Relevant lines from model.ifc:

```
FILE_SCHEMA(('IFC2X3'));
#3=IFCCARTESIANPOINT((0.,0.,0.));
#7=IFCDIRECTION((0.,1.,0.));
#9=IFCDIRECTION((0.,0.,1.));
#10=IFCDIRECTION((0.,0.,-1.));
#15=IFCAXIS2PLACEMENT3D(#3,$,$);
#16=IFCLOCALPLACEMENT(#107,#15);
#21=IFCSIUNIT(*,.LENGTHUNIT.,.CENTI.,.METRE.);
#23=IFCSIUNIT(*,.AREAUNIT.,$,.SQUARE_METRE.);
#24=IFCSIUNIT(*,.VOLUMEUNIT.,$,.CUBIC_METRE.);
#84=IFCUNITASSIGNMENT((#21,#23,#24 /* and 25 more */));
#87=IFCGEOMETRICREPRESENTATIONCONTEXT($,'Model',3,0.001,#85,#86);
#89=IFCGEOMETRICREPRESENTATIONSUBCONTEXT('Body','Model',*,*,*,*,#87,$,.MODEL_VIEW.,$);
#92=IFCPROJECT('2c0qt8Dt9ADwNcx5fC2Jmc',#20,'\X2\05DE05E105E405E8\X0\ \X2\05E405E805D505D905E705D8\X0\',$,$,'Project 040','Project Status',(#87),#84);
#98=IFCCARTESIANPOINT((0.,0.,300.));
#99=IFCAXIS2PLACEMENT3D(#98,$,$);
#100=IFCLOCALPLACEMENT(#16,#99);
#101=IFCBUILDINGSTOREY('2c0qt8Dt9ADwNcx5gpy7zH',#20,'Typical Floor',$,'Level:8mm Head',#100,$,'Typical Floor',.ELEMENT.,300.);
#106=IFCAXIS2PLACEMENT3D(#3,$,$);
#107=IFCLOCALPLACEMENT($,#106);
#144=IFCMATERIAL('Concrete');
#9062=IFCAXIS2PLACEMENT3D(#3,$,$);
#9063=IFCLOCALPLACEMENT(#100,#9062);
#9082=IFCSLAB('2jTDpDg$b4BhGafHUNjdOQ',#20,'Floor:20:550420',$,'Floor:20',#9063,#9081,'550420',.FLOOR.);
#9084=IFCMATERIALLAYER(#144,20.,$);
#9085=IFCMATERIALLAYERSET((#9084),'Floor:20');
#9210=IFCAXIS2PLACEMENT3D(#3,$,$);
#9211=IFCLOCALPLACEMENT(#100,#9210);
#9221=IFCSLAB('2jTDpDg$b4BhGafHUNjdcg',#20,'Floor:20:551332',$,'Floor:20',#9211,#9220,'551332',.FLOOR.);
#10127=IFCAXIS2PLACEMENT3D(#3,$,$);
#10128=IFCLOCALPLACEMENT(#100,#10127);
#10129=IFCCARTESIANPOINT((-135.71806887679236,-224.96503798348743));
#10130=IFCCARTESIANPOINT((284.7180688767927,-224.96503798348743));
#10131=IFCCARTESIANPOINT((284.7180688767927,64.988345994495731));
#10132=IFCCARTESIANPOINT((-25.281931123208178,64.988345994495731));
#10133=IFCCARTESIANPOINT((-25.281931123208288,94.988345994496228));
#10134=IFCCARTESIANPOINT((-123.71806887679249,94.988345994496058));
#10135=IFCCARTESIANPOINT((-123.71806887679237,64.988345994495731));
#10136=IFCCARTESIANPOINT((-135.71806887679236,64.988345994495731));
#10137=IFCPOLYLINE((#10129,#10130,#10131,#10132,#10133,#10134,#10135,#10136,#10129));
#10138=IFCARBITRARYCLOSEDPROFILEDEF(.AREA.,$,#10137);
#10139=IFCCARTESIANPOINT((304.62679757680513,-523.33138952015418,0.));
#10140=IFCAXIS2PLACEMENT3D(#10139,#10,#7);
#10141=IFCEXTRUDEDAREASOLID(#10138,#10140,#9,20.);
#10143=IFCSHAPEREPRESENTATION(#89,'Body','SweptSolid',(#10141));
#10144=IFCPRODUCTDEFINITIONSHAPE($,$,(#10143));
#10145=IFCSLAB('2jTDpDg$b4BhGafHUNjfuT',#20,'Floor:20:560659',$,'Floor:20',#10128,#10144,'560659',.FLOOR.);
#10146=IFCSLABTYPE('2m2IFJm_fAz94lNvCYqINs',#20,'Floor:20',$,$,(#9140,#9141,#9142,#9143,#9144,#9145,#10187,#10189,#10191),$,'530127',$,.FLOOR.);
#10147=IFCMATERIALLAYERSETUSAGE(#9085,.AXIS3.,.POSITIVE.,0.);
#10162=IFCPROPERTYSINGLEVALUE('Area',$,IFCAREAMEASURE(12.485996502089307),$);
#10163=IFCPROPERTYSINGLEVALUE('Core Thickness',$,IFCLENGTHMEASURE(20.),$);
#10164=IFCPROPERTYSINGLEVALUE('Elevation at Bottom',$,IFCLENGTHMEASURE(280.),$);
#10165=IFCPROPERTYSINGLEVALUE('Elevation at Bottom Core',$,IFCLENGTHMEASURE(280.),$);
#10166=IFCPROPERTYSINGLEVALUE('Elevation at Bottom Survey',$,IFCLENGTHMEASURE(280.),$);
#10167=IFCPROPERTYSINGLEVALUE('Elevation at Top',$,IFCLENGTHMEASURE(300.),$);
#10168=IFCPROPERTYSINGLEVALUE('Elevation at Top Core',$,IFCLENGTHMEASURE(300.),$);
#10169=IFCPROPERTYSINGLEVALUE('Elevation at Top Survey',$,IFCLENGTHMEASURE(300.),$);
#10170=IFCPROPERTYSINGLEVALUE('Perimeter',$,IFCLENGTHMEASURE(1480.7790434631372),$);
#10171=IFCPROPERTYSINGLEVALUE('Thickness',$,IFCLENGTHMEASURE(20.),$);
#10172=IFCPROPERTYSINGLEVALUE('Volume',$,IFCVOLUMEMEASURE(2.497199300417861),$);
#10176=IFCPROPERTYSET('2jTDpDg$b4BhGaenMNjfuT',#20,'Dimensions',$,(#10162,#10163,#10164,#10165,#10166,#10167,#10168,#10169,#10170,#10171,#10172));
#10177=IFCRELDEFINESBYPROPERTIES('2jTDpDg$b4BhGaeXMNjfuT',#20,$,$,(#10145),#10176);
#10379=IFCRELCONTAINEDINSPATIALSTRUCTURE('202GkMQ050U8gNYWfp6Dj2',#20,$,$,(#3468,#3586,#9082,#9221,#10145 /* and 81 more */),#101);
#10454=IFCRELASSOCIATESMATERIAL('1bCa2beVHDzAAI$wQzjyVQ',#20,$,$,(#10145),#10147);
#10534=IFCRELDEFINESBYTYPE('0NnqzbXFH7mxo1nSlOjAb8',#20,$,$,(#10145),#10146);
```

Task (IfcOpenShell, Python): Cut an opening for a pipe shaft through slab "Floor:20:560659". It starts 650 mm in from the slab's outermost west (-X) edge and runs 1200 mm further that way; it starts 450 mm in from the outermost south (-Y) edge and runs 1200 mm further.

```python
import numpy as np
import ifcopenshell
import ifcopenshell.api.feature
import ifcopenshell.api.geometry
import ifcopenshell.api.pset
import ifcopenshell.api.root
import ifcopenshell.geom
import ifcopenshell.util.element
import ifcopenshell.util.placement
import ifcopenshell.util.representation
import ifcopenshell.util.shape
import ifcopenshell.util.unit

model = ifcopenshell.open("model.ifc")
unit_scale = ifcopenshell.util.unit.calculate_unit_scale(model)
area_scale = ifcopenshell.util.unit.calculate_unit_scale(model, "AREAUNIT")
volume_scale = ifcopenshell.util.unit.calculate_unit_scale(model, "VOLUMEUNIT")
settings = ifcopenshell.geom.settings()


def volume(element):
    """Net volume in cubic metres, openings subtracted."""
    shape = ifcopenshell.geom.create_shape(settings, element)
    return ifcopenshell.util.shape.get_volume(shape.geometry)


slab = model.by_guid("2jTDpDg$b4BhGafHUNjfuT")
before = volume(slab)

# Extent in the slab's own axes, in metres. The edges named are its -X and -Y sides.
slab_shape = ifcopenshell.geom.create_shape(settings, slab)
vertices = ifcopenshell.util.shape.get_vertices(slab_shape.geometry)
x_min, y_min, bottom = vertices.min(axis=0)
top = vertices[:, 2].max()

opening = ifcopenshell.api.root.create_entity(model, ifc_class="IfcOpeningElement", name="Pipe shaft opening")
context = ifcopenshell.util.representation.get_context(model, "Model", "Body", "MODEL_VIEW")
width, depth = 1.2, 1.2
outline = [(0.0, 0.0), (width, 0.0), (width, depth), (0.0, depth), (0.0, 0.0)]
# Overshoot both faces by 50 mm so the cut is clean.
shape = ifcopenshell.api.geometry.add_slab_representation(
    model, context=context, depth=top - bottom + 0.1, polyline=outline
)
ifcopenshell.api.geometry.assign_representation(model, product=opening, representation=shape)

matrix = ifcopenshell.util.placement.get_local_placement(slab.ObjectPlacement)
matrix[:, 3] = matrix @ np.append(np.array([x_min + 0.65, y_min + 0.45, bottom - 0.05]) / unit_scale, 1.0)
ifcopenshell.api.geometry.edit_object_placement(model, product=opening, matrix=matrix, is_si=False)
ifcopenshell.api.feature.add_feature(model, feature=opening, element=slab)

after = volume(slab)

# Update the slab's stored quantities.
pset = model.by_id(ifcopenshell.util.element.get_pset(slab, "Dimensions", should_inherit=False)["id"])
ifcopenshell.api.pset.edit_pset(model, pset=pset, properties={
    "Area": model.create_entity("IfcAreaMeasure", after / (top - bottom) / area_scale),
    "Volume": model.create_entity("IfcVolumeMeasure", after / volume_scale),
})

print(f"slab volume {before:.3f} -> {after:.3f} m3")

model.write("model_edited.ifc")
```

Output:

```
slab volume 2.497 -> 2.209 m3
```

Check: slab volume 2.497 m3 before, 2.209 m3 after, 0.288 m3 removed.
